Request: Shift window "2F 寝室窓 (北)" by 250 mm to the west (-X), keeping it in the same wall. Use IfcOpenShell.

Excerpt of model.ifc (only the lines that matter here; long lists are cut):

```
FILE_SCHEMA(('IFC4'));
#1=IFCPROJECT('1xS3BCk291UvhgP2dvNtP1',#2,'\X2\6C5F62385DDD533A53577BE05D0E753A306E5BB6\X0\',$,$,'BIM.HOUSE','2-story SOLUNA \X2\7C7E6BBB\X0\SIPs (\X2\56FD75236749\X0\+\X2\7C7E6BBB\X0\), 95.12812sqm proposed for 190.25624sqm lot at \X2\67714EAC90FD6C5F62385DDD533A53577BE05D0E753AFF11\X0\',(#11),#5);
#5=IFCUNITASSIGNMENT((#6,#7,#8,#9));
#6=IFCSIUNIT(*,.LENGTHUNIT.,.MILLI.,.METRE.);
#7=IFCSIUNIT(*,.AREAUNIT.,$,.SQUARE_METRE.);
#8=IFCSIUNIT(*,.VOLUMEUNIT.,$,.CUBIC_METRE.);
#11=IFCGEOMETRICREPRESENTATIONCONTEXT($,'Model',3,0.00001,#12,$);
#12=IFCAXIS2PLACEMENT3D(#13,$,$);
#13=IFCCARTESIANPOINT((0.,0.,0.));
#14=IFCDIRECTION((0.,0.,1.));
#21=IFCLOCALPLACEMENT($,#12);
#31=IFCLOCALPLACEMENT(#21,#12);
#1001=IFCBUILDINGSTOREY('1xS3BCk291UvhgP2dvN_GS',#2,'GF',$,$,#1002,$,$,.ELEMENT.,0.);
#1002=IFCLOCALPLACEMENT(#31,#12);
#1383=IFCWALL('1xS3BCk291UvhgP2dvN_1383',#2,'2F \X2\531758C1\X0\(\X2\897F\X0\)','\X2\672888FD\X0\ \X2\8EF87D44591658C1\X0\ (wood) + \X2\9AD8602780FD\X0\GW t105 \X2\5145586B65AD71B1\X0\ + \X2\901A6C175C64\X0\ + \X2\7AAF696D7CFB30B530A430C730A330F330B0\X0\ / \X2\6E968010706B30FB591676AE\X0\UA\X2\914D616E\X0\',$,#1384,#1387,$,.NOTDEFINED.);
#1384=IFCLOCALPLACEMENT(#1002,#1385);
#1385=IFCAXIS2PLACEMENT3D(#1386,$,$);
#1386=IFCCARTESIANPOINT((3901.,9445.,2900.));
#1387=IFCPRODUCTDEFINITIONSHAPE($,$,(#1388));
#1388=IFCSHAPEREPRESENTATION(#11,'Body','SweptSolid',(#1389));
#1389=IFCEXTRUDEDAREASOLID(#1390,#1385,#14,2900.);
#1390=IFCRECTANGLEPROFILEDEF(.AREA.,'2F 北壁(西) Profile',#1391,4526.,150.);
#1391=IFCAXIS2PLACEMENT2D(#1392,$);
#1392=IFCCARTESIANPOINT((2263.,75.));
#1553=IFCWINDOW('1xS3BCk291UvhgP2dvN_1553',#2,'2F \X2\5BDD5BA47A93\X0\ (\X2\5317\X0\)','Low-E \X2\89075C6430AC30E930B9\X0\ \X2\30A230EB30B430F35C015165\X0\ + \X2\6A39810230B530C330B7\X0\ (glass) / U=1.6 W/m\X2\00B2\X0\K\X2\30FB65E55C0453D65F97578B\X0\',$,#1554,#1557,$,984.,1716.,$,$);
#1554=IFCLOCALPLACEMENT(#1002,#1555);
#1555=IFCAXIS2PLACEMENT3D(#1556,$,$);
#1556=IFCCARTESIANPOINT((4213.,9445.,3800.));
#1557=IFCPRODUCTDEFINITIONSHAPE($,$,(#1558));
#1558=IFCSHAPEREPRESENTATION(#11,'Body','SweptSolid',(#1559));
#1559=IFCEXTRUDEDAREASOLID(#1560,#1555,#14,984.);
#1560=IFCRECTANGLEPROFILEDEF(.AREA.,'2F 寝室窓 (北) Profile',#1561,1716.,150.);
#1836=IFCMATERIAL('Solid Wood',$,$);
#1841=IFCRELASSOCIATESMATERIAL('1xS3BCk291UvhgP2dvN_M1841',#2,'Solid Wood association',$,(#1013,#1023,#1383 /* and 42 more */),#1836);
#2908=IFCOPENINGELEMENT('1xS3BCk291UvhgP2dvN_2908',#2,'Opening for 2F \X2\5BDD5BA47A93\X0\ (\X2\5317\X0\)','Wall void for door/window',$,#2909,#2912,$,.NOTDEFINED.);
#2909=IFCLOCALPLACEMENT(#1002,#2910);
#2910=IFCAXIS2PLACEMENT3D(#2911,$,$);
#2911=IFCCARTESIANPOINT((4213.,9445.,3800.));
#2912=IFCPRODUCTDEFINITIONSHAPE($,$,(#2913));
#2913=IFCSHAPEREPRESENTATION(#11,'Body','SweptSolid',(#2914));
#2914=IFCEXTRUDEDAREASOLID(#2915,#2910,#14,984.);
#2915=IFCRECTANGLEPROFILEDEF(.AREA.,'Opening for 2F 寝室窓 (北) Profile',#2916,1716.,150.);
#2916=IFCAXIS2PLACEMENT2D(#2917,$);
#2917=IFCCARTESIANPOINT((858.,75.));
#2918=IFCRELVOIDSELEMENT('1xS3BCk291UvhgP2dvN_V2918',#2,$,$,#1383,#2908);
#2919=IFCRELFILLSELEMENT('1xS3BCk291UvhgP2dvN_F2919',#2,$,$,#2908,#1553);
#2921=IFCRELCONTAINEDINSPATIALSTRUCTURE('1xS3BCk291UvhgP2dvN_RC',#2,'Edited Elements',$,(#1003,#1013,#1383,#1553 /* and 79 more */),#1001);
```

```python
import ifcopenshell
import ifcopenshell.api.geometry
import ifcopenshell.util.placement

model = ifcopenshell.open("model.ifc")

window = model.by_guid("1xS3BCk291UvhgP2dvN_1553")
opening = window.FillsVoids[0].RelatingOpeningElement
wall = opening.VoidsElements[0].RelatingBuildingElement

wall_matrix = ifcopenshell.util.placement.get_local_placement(wall.ObjectPlacement)
shift = wall_matrix[:3, 0] * -250.0
before = ifcopenshell.util.placement.get_local_placement(window.ObjectPlacement)[:3, 3].copy()

# The window is not placed relative to its opening, so move both.
for product in (opening, window):
    matrix = ifcopenshell.util.placement.get_local_placement(product.ObjectPlacement)
    matrix[:3, 3] += shift
    ifcopenshell.api.geometry.edit_object_placement(model, product=product, matrix=matrix, is_si=False)

after = ifcopenshell.util.placement.get_local_placement(window.ObjectPlacement)[:3, 3]
print("window moved by", (after - before).round(3) + 0.0)

model.write("model_edited.ifc")
```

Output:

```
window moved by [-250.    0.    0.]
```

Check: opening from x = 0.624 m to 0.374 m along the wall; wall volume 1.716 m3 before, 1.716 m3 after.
